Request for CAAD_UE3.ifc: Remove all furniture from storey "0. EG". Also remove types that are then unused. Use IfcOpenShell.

First a look at what the model holds.

```python
import ifcopenshell
import ifcopenshell.util.element

model = ifcopenshell.open("CAAD_UE3.ifc")
print(model.schema)
storey = next(s for s in model.by_type("IfcBuildingStorey") if s.Name == "0. EG")
furniture = [e for e in ifcopenshell.util.element.get_decomposition(storey) if e.is_a("IfcFurnishingElement")]
seen = {}
for e in furniture:
    element_type = ifcopenshell.util.element.get_type(e)
    name = element_type.Name if element_type not in (None, e) else None
    seen[name] = seen.get(name, 0) + 1
for name, count in sorted(seen.items(), key=str):
    print(count, "x", name)
```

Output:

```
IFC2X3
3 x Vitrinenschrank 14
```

```python
import ifcopenshell
import ifcopenshell.api.root
import ifcopenshell.util.element

model = ifcopenshell.open("CAAD_UE3.ifc")

storey = next(s for s in model.by_type("IfcBuildingStorey") if s.Name == "0. EG")
furniture = [e for e in ifcopenshell.util.element.get_decomposition(storey) if e.is_a("IfcFurnishingElement")]
types = {ifcopenshell.util.element.get_type(e) for e in furniture} - {None, *furniture}

for e in furniture:
    ifcopenshell.api.root.remove_product(model, product=e)
print(len(furniture), "removed")

unused = [t for t in types if not ifcopenshell.util.element.get_types(t)]
for t in unused:
    ifcopenshell.api.root.remove_product(model, product=t)
print(len(unused), "unused types removed")

model.write("CAAD_UE3_rev.ifc")
```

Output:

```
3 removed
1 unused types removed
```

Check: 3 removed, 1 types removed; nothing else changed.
